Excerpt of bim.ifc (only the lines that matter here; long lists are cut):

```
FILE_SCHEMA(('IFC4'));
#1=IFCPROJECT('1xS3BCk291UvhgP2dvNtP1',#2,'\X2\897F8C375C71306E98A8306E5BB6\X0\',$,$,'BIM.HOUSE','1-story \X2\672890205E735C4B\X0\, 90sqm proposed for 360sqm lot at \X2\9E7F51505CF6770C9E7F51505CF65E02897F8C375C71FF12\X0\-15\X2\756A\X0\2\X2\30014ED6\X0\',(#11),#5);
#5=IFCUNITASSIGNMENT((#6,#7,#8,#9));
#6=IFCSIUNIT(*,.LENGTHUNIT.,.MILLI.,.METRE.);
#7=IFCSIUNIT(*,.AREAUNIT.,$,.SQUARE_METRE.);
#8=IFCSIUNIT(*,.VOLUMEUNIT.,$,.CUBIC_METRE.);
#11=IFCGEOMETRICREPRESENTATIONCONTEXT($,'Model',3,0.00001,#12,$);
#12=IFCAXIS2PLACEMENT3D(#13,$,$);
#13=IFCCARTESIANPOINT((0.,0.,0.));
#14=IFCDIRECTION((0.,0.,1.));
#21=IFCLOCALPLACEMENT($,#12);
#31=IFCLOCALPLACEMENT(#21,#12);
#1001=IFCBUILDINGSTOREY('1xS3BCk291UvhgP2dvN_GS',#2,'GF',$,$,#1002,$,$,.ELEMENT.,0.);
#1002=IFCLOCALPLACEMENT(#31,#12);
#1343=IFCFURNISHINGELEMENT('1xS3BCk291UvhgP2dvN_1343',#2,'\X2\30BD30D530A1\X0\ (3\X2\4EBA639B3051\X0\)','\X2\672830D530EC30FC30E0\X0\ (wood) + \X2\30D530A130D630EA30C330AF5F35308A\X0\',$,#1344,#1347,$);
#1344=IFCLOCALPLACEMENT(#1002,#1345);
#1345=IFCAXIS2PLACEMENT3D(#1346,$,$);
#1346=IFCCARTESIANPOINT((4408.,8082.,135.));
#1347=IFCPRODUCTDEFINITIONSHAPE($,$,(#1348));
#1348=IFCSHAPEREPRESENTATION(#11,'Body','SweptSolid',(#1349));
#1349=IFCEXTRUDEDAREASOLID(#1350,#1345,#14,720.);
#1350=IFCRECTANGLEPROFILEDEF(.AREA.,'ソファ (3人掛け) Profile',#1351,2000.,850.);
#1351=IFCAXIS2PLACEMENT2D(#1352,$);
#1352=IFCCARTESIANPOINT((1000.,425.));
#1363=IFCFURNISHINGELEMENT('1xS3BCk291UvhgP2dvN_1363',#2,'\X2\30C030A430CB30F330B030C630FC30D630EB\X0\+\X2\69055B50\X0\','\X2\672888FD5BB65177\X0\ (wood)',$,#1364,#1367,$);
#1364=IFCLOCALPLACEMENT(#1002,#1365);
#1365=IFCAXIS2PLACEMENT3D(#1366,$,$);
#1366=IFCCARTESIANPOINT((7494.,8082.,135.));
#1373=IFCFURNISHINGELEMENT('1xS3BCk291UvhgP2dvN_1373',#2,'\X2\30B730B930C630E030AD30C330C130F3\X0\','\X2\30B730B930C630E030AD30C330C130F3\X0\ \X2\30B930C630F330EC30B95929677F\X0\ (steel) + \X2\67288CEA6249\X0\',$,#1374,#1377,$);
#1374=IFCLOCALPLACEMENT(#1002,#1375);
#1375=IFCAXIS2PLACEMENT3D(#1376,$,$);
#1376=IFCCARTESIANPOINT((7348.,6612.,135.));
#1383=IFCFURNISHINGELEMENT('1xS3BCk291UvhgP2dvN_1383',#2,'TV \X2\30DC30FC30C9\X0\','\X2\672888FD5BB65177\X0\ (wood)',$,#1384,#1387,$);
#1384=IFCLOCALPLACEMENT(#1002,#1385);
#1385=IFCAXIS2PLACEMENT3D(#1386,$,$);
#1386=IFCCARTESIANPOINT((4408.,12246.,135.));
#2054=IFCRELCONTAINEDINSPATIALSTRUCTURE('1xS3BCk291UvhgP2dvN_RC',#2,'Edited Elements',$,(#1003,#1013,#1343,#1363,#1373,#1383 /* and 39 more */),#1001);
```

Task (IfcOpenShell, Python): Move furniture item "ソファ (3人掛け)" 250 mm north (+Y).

```python
import ifcopenshell
import ifcopenshell.api.geometry
import ifcopenshell.util.placement

model = ifcopenshell.open("bim.ifc")

item = model.by_guid("1xS3BCk291UvhgP2dvN_1343")
matrix = ifcopenshell.util.placement.get_local_placement(item.ObjectPlacement)
matrix[1, 3] += 250.0
ifcopenshell.api.geometry.edit_object_placement(model, product=item, matrix=matrix, is_si=False)

print(ifcopenshell.util.placement.get_local_placement(item.ObjectPlacement).round(3) + 0.0)

model.write("bim_rev.ifc")
```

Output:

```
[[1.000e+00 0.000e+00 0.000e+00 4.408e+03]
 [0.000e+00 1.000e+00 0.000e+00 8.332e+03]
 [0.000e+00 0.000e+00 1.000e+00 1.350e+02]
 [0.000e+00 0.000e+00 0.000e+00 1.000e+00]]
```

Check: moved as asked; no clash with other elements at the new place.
